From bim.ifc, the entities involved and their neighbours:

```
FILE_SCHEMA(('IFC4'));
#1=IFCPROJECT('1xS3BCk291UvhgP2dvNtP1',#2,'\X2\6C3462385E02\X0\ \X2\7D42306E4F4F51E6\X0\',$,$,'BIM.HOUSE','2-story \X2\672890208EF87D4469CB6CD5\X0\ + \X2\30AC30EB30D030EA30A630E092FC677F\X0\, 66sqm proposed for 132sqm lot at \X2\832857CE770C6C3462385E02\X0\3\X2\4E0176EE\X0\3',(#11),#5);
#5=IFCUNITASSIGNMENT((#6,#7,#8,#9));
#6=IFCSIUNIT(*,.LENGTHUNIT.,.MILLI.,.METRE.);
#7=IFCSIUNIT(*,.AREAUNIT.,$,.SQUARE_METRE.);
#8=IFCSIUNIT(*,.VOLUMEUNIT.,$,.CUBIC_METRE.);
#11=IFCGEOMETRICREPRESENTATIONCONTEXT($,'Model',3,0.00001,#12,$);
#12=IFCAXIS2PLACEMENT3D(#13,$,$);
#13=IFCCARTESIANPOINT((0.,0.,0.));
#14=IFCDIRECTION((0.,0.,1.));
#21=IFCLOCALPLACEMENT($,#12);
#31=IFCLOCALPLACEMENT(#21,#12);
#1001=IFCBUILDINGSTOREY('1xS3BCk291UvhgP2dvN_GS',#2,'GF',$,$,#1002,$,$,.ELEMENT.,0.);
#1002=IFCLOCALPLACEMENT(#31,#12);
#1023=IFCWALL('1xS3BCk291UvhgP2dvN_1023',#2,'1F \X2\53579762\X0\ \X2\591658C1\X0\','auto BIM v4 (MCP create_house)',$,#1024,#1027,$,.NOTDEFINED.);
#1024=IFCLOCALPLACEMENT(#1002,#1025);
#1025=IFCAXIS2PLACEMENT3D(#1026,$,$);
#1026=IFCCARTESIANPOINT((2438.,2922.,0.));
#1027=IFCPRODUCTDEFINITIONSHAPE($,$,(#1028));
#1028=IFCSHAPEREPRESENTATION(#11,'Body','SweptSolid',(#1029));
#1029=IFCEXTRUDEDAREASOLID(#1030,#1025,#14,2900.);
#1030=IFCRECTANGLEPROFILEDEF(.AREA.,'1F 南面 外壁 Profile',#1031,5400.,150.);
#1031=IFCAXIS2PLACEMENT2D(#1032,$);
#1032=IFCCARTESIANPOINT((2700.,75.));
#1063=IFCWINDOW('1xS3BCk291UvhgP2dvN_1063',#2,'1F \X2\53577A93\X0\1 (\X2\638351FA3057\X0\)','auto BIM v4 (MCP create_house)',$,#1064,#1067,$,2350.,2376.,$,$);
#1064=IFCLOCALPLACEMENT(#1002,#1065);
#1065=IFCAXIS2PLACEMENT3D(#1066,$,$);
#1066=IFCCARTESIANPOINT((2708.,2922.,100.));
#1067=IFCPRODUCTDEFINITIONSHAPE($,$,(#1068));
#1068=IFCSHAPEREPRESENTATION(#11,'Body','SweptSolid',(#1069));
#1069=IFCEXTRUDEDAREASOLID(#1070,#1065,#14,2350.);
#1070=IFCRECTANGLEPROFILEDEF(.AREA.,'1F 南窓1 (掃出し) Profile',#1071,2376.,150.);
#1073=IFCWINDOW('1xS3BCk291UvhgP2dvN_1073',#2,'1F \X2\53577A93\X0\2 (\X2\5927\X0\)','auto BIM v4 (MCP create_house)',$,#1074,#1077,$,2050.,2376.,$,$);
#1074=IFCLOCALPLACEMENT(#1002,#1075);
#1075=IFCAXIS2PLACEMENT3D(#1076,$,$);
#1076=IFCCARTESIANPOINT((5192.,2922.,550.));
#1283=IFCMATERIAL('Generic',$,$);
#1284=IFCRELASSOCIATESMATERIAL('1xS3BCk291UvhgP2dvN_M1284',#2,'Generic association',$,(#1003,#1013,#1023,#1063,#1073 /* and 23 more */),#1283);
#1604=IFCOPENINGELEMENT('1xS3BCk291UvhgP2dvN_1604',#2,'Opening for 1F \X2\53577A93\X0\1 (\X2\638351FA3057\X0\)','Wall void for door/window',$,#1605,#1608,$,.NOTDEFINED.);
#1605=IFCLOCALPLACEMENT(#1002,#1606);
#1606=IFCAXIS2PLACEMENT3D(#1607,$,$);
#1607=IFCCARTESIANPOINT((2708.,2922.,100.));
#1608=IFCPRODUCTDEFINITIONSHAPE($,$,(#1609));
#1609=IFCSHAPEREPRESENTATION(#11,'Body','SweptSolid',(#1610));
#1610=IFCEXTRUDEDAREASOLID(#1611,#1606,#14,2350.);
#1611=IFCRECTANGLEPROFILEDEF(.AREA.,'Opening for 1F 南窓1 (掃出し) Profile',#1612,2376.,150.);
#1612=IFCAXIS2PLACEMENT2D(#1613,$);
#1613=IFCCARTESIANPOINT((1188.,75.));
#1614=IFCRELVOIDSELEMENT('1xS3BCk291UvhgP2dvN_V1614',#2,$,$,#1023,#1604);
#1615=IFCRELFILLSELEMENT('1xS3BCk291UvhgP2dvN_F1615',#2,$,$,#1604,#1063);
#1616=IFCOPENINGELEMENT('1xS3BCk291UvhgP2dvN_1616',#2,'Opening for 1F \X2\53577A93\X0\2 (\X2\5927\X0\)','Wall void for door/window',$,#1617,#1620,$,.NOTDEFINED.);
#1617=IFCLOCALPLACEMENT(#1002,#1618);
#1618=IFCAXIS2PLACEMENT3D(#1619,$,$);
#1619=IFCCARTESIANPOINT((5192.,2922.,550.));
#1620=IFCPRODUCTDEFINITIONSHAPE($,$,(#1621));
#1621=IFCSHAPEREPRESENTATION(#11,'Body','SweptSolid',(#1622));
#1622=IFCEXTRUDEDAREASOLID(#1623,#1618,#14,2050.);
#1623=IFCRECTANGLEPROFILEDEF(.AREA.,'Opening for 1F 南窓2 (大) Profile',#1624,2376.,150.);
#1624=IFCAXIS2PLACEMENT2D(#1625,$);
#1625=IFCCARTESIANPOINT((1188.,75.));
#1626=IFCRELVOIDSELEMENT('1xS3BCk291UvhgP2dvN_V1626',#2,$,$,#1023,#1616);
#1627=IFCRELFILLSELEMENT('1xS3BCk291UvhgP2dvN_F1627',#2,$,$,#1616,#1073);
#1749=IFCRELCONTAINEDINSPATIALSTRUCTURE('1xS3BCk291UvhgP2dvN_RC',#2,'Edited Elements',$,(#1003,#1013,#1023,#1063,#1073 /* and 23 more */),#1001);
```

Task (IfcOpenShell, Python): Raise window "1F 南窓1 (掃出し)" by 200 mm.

```python
import numpy as np
import ifcopenshell
import ifcopenshell.api.geometry
import ifcopenshell.util.placement
import ifcopenshell.util.unit

model = ifcopenshell.open("bim.ifc")
unit_scale = ifcopenshell.util.unit.calculate_unit_scale(model)

window = model.by_id(1063)
opening = window.FillsVoids[0].RelatingOpeningElement
dz = 200.0

shift = np.array([0.0, 0.0, dz])
# The window is not placed relative to its opening, so move both.
for product in (opening, window):
    matrix = ifcopenshell.util.placement.get_local_placement(product.ObjectPlacement)
    matrix[:3, 3] += shift
    ifcopenshell.api.geometry.edit_object_placement(model, product=product, matrix=matrix, is_si=False)

print(f"moved by {dz * unit_scale:+.3f} m")

model.write("bim_v2.ifc")
```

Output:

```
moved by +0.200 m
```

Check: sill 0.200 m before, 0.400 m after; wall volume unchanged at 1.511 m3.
